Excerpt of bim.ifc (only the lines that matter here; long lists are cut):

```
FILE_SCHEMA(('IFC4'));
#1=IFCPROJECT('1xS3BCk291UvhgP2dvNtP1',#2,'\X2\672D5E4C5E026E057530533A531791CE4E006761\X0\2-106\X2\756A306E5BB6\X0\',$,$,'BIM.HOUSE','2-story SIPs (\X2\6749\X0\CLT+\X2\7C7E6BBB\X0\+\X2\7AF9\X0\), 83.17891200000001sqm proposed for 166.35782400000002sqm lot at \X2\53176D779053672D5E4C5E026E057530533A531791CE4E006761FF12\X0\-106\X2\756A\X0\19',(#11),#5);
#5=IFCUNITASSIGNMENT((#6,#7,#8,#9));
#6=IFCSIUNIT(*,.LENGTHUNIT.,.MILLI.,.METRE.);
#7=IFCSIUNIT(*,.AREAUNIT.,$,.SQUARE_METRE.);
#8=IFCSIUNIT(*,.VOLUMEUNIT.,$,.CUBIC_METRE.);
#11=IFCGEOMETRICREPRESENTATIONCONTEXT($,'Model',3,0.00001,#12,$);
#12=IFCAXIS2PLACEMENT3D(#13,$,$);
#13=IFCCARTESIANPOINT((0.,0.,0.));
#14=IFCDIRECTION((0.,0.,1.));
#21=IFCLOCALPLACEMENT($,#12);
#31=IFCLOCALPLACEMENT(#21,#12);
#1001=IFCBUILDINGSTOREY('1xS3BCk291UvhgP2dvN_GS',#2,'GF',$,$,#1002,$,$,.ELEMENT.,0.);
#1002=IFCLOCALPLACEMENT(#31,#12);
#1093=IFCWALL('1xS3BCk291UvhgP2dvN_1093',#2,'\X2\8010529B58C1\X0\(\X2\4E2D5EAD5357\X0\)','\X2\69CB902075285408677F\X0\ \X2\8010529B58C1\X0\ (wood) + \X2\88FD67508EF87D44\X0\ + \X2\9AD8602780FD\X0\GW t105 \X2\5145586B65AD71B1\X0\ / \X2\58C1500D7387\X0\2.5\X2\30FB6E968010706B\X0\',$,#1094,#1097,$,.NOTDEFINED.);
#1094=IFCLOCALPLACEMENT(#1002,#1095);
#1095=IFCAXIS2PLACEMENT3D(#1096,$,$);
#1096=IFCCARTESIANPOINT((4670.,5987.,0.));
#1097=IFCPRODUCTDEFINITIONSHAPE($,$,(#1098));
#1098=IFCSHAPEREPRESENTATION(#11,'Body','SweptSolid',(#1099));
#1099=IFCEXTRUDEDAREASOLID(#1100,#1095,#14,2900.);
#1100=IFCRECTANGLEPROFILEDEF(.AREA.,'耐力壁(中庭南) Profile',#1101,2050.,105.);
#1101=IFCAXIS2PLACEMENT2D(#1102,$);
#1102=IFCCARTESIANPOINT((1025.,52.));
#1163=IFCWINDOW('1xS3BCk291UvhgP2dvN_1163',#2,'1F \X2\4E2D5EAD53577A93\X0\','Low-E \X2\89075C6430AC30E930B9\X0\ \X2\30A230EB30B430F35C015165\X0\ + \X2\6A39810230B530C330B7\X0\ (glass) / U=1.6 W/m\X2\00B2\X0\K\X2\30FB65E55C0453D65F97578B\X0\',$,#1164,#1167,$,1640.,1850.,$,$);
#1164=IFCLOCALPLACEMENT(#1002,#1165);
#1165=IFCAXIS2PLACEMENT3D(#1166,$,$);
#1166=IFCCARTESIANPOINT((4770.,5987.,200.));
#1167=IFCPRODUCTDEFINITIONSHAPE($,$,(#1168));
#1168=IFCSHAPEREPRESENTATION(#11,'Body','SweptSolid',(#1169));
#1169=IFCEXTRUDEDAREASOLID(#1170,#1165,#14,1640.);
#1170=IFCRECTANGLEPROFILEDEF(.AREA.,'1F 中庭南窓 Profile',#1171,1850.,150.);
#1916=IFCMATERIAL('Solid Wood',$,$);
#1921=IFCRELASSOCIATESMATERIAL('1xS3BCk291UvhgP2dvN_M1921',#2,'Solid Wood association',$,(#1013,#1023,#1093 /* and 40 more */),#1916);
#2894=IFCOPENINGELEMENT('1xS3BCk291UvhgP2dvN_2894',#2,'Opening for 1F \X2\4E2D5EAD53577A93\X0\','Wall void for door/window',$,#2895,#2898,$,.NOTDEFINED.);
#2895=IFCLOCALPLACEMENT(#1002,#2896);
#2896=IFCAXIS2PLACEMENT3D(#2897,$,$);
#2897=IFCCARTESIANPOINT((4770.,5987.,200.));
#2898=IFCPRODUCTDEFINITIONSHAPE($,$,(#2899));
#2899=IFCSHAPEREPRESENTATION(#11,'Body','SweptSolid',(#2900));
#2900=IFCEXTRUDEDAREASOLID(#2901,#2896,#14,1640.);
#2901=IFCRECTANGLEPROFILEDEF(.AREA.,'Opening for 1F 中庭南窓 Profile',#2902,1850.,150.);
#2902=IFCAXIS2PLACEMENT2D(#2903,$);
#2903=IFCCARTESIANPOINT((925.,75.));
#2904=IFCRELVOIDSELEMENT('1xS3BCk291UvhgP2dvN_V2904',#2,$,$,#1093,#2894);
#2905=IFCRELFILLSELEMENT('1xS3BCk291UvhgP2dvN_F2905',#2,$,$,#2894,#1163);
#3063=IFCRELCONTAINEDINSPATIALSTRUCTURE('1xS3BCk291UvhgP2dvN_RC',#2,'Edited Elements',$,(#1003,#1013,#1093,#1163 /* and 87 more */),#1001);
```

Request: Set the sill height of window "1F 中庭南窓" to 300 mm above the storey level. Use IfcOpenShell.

```python
import numpy as np
import ifcopenshell
import ifcopenshell.api.geometry
import ifcopenshell.geom
import ifcopenshell.util.element
import ifcopenshell.util.placement
import ifcopenshell.util.shape
import ifcopenshell.util.unit

model = ifcopenshell.open("bim.ifc")
unit_scale = ifcopenshell.util.unit.calculate_unit_scale(model)

window = model.by_guid("1xS3BCk291UvhgP2dvN_1163")
opening = window.FillsVoids[0].RelatingOpeningElement
storey = ifcopenshell.util.element.get_container(window, ifc_class="IfcBuildingStorey")
level = ifcopenshell.util.placement.get_local_placement(storey.ObjectPlacement)[2, 3]

# The opening's origin need not be at the sill, so measure its lowest point.
shape = ifcopenshell.geom.create_shape(ifcopenshell.geom.settings(), opening)
bottom = ifcopenshell.util.shape.get_shape_bottom_elevation(shape, shape.geometry) / unit_scale
dz = level + 0.3 / unit_scale - bottom

shift = np.array([0.0, 0.0, dz])
# The window is not placed relative to its opening, so move both.
for product in (opening, window):
    matrix = ifcopenshell.util.placement.get_local_placement(product.ObjectPlacement)
    matrix[:3, 3] += shift
    ifcopenshell.api.geometry.edit_object_placement(model, product=product, matrix=matrix, is_si=False)

print(f"moved by {dz * unit_scale:+.3f} m")

model.write("bim_v2.ifc")
```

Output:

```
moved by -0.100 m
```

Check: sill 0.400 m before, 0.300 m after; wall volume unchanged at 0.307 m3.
